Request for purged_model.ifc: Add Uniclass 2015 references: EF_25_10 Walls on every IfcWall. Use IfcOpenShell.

First a look at what the model holds.

```python
import ifcopenshell

model = ifcopenshell.open("purged_model.ifc")
print(model.schema)
print("classifications:", [c.Name for c in model.by_type("IfcClassification")])
for ifc_class in ("IfcDoor", "IfcRoof", "IfcStair", "IfcWall", "IfcWindow"):
    print(ifc_class, len(model.by_type(ifc_class)))
```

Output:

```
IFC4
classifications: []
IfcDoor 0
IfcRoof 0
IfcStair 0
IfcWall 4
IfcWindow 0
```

```python
import ifcopenshell
import ifcopenshell.api.classification

model = ifcopenshell.open("purged_model.ifc")

system = ifcopenshell.api.classification.add_classification(model, classification="Uniclass 2015")

codes = {
    "IfcWall": ("EF_25_10", "Walls"),
}
for ifc_class, (code, name) in codes.items():
    products = model.by_type(ifc_class)
    ifcopenshell.api.classification.add_reference(
        model, products=products, classification=system, identification=code, name=name
    )
    print(code, len(products))

model.write("purged_model_v2.ifc")
```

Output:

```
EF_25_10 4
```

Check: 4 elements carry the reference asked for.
